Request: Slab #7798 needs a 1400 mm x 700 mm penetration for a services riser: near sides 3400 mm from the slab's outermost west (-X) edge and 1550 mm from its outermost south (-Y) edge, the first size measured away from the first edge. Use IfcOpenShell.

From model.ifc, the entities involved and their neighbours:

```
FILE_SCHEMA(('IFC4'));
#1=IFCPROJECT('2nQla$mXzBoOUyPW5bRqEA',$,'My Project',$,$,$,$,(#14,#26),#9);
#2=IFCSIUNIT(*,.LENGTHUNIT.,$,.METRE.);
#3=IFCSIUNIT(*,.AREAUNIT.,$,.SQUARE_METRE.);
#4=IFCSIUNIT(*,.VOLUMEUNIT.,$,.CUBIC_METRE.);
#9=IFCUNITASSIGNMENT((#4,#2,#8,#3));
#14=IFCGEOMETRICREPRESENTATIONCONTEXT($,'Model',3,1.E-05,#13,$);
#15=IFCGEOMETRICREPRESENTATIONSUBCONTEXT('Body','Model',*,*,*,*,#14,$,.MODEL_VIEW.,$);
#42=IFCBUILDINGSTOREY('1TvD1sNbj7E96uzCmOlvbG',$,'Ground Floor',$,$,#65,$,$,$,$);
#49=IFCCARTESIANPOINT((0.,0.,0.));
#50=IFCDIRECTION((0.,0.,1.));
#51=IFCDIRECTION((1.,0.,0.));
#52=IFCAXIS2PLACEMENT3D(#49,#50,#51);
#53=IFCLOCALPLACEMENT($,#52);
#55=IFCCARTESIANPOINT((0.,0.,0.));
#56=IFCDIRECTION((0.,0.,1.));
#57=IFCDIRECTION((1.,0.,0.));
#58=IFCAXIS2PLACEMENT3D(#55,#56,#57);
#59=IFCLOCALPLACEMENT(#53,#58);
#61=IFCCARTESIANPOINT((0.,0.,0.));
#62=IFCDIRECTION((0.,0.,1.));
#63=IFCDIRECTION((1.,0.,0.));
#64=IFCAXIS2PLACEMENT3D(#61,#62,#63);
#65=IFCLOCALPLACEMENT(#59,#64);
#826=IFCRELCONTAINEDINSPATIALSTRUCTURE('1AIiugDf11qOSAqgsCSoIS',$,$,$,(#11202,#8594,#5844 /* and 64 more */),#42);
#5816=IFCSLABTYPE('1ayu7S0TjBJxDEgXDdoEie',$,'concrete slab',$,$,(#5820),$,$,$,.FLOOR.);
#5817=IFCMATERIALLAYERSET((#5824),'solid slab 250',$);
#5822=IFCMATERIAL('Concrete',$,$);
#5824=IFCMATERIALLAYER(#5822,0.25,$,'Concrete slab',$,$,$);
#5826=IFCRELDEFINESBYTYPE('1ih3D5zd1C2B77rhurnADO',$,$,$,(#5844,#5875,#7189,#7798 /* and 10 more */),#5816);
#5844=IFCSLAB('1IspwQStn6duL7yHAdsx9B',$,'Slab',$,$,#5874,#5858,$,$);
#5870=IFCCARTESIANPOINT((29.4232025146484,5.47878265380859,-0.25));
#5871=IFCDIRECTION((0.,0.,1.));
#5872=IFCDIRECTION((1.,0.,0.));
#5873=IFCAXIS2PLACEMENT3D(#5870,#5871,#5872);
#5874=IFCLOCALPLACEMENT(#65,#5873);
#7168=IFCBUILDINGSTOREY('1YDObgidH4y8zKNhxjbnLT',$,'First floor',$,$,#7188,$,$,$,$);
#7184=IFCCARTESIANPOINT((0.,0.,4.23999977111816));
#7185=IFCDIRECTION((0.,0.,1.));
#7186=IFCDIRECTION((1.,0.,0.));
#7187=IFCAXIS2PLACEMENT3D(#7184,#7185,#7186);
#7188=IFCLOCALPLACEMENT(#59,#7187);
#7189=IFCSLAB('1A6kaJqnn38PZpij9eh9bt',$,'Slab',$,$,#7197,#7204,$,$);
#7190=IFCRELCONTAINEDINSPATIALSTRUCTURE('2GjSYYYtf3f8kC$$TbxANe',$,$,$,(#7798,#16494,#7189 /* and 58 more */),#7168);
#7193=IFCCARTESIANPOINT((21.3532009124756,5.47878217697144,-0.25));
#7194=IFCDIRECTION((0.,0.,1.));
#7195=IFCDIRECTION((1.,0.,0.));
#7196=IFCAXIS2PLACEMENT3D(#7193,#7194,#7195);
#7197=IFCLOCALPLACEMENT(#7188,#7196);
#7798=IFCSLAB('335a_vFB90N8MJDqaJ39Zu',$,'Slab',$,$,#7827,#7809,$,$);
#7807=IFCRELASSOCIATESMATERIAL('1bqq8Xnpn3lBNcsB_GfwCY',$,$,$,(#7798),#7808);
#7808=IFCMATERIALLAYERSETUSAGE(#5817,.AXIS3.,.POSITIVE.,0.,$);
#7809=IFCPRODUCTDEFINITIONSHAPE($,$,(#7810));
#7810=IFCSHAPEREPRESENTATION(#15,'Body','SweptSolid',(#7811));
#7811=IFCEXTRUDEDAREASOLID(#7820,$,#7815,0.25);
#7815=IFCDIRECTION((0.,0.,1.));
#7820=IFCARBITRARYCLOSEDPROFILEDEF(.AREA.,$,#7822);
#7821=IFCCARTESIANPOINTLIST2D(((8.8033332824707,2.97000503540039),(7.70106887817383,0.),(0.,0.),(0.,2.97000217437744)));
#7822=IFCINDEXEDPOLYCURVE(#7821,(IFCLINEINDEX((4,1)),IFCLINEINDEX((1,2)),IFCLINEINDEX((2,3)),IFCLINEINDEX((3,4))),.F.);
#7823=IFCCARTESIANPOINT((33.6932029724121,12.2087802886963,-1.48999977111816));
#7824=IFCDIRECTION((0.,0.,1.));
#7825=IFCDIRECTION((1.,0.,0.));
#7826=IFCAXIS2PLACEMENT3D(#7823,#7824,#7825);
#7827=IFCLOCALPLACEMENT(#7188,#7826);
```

```python
import numpy as np
import ifcopenshell
import ifcopenshell.api.feature
import ifcopenshell.api.geometry
import ifcopenshell.api.root
import ifcopenshell.geom
import ifcopenshell.util.placement
import ifcopenshell.util.representation
import ifcopenshell.util.shape
import ifcopenshell.util.unit

model = ifcopenshell.open("model.ifc")
unit_scale = ifcopenshell.util.unit.calculate_unit_scale(model)
settings = ifcopenshell.geom.settings()


def volume(element):
    """Net volume in cubic metres, openings subtracted."""
    shape = ifcopenshell.geom.create_shape(settings, element)
    return ifcopenshell.util.shape.get_volume(shape.geometry)


slab = model.by_id(7798)
before = volume(slab)

# Extent in the slab's own axes, in metres. The edges named are its -X and -Y sides.
slab_shape = ifcopenshell.geom.create_shape(settings, slab)
vertices = ifcopenshell.util.shape.get_vertices(slab_shape.geometry)
x_min, y_min, bottom = vertices.min(axis=0)
top = vertices[:, 2].max()

opening = ifcopenshell.api.root.create_entity(model, ifc_class="IfcOpeningElement", name="Services riser opening", predefined_type="OPENING")
context = ifcopenshell.util.representation.get_context(model, "Model", "Body", "MODEL_VIEW")
width, depth = 1.4, 0.7
outline = [(0.0, 0.0), (width, 0.0), (width, depth), (0.0, depth), (0.0, 0.0)]
# Overshoot both faces by 50 mm so the cut is clean.
shape = ifcopenshell.api.geometry.add_slab_representation(
    model, context=context, depth=top - bottom + 0.1, polyline=outline
)
ifcopenshell.api.geometry.assign_representation(model, product=opening, representation=shape)

matrix = ifcopenshell.util.placement.get_local_placement(slab.ObjectPlacement)
matrix[:, 3] = matrix @ np.append(np.array([x_min + 3.4, y_min + 1.55, bottom - 0.05]) / unit_scale, 1.0)
ifcopenshell.api.geometry.edit_object_placement(model, product=opening, matrix=matrix, is_si=False)
ifcopenshell.api.feature.add_feature(model, feature=opening, element=slab)

after = volume(slab)

print(f"slab volume {before:.3f} -> {after:.3f} m3")

model.write("model_edited.ifc")
```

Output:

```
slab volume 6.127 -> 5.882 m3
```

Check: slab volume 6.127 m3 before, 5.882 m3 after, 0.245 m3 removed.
